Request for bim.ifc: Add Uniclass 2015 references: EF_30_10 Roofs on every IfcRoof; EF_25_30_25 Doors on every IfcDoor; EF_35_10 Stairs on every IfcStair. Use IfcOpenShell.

First a look at what the model holds.

```python
import ifcopenshell

model = ifcopenshell.open("bim.ifc")
print(model.schema)
print("classifications:", [c.Name for c in model.by_type("IfcClassification")])
for ifc_class in ("IfcDoor", "IfcRoof", "IfcStair", "IfcWall", "IfcWindow"):
    print(ifc_class, len(model.by_type(ifc_class)))
```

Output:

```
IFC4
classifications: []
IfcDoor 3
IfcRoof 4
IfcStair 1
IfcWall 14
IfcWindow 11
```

```python
import ifcopenshell
import ifcopenshell.api.classification

model = ifcopenshell.open("bim.ifc")

system = ifcopenshell.api.classification.add_classification(model, classification="Uniclass 2015")

codes = {
    "IfcRoof": ("EF_30_10", "Roofs"),
    "IfcDoor": ("EF_25_30_25", "Doors"),
    "IfcStair": ("EF_35_10", "Stairs"),
}
for ifc_class, (code, name) in codes.items():
    products = model.by_type(ifc_class)
    ifcopenshell.api.classification.add_reference(
        model, products=products, classification=system, identification=code, name=name
    )
    print(code, len(products))

model.write("bim-out.ifc")
```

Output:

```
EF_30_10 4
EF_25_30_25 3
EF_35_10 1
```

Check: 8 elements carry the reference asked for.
